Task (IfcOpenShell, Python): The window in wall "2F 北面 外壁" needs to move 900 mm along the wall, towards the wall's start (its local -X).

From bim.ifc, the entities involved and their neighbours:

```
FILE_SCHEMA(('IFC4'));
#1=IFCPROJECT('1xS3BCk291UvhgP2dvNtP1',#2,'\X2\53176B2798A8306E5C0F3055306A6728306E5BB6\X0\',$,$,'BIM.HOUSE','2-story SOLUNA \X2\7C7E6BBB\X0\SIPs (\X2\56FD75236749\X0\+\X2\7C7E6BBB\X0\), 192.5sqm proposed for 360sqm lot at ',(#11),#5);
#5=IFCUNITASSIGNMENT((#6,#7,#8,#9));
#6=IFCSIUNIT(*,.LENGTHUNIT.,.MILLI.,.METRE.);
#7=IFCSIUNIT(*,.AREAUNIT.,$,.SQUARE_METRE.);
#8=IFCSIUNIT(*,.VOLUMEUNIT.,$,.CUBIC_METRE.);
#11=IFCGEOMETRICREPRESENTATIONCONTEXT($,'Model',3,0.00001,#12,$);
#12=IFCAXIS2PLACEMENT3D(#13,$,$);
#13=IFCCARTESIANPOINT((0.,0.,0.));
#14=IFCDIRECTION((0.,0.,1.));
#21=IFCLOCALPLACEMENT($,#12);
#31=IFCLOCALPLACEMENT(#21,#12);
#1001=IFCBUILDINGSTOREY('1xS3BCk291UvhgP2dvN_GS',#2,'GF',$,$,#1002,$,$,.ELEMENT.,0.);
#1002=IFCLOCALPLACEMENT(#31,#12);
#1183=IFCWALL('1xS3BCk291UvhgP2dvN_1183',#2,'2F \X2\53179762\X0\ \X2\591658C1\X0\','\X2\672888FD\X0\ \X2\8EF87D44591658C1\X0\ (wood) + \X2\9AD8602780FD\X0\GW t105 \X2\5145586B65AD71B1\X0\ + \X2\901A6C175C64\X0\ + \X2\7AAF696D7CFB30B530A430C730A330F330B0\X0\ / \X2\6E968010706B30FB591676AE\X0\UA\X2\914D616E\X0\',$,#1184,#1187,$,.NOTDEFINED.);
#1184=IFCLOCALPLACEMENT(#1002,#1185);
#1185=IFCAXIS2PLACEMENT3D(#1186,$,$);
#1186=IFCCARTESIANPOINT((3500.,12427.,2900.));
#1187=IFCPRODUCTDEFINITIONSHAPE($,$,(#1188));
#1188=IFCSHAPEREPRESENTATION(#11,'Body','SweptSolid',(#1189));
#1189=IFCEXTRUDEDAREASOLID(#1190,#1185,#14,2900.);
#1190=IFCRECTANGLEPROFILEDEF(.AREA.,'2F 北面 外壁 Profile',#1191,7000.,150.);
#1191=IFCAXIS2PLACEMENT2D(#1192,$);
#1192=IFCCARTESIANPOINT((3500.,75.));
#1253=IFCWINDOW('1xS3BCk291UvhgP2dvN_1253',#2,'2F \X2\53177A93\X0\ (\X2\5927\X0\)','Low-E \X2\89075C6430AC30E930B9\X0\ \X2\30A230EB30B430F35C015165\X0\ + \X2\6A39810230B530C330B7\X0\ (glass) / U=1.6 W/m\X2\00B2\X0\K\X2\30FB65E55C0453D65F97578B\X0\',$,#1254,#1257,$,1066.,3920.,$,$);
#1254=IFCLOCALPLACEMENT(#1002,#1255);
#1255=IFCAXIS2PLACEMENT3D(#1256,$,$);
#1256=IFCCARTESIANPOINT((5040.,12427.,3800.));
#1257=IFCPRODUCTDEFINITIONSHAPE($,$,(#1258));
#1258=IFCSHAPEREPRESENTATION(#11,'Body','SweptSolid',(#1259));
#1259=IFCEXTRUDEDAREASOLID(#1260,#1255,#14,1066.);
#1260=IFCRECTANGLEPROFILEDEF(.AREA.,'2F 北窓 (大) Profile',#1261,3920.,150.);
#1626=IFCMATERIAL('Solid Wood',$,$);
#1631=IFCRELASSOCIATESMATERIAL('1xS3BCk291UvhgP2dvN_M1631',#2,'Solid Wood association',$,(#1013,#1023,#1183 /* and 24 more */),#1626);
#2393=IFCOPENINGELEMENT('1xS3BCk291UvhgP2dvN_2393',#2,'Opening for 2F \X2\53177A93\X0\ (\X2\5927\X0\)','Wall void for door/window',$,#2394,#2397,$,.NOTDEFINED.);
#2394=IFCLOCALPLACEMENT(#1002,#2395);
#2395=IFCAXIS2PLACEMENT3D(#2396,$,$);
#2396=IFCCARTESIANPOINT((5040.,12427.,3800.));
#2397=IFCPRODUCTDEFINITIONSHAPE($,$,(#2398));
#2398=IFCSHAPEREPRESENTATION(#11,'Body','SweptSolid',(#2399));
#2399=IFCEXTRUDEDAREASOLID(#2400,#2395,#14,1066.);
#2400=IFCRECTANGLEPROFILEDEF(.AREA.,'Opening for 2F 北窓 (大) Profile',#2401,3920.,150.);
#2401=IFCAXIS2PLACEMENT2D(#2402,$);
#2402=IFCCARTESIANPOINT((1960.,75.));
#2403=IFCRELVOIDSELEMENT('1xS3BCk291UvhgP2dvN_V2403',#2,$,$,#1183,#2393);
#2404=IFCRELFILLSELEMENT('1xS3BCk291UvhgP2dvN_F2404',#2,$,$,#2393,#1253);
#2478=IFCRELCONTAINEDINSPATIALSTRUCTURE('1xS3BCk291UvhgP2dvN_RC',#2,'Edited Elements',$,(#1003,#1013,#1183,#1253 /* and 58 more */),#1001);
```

```python
import ifcopenshell
import ifcopenshell.api.geometry
import ifcopenshell.util.placement

model = ifcopenshell.open("bim.ifc")

window = model.by_guid("1xS3BCk291UvhgP2dvN_1253")
opening = window.FillsVoids[0].RelatingOpeningElement
wall = opening.VoidsElements[0].RelatingBuildingElement

wall_matrix = ifcopenshell.util.placement.get_local_placement(wall.ObjectPlacement)
shift = wall_matrix[:3, 0] * -900.0
before = ifcopenshell.util.placement.get_local_placement(window.ObjectPlacement)[:3, 3].copy()

# The window is not placed relative to its opening, so move both.
for product in (opening, window):
    matrix = ifcopenshell.util.placement.get_local_placement(product.ObjectPlacement)
    matrix[:3, 3] += shift
    ifcopenshell.api.geometry.edit_object_placement(model, product=product, matrix=matrix, is_si=False)

after = ifcopenshell.util.placement.get_local_placement(window.ObjectPlacement)[:3, 3]
print("window moved by", (after - before).round(3) + 0.0)

model.write("bim_rev.ifc")
```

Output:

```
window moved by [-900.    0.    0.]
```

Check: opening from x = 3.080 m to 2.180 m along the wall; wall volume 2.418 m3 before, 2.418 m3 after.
